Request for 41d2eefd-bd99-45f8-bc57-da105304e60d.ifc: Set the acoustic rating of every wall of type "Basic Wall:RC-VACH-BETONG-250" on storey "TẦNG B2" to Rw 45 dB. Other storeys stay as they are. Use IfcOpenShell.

First a look at what the model holds.

```python
import ifcopenshell
import ifcopenshell.util.element

model = ifcopenshell.open("41d2eefd-bd99-45f8-bc57-da105304e60d.ifc")
print(model.schema)
storey = next(s for s in model.by_type("IfcBuildingStorey") if s.Name == "TẦNG B2")
walls = [e for e in ifcopenshell.util.element.get_decomposition(storey) if e.is_a("IfcWall")]
seen = {}
for e in walls:
    element_type = ifcopenshell.util.element.get_type(e)
    key = (element_type.Name if element_type != e and element_type else None, ifcopenshell.util.element.get_pset(e, "Pset_WallCommon", "AcousticRating"))
    seen[key] = seen.get(key, 0) + 1
for (name, value), count in sorted(seen.items(), key=str):
    print(count, "x", name, "|", value)
```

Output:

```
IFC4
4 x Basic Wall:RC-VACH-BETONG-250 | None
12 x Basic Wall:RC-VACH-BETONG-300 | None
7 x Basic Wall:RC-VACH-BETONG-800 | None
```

```python
import ifcopenshell
import ifcopenshell.api.pset
import ifcopenshell.util.element

model = ifcopenshell.open("41d2eefd-bd99-45f8-bc57-da105304e60d.ifc")

storey = next(s for s in model.by_type("IfcBuildingStorey") if s.Name == "TẦNG B2")
walls = [e for e in ifcopenshell.util.element.get_decomposition(storey) if e.is_a("IfcWall")]

count = 0
for e in walls:
    element_type = ifcopenshell.util.element.get_type(e)
    if element_type in (None, e) or element_type.Name != "Basic Wall:RC-VACH-BETONG-250":
        continue
    # add_pset returns the element's existing set when there is one.
    pset = ifcopenshell.api.pset.add_pset(model, product=e, name="Pset_WallCommon")
    ifcopenshell.api.pset.edit_pset(model, pset=pset, properties={"AcousticRating": "Rw 45 dB"})
    count += 1

print(count, "walls updated")

model.write("41d2eefd-bd99-45f8-bc57-da105304e60d_edited.ifc")
```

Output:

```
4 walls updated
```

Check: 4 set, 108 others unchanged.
